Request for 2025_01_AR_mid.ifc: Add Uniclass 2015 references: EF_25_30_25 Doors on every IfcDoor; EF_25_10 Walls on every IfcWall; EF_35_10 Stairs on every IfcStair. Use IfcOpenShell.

First a look at what the model holds.

```python
import ifcopenshell

model = ifcopenshell.open("2025_01_AR_mid.ifc")
print(model.schema)
print("classifications:", [c.Name for c in model.by_type("IfcClassification")])
for ifc_class in ("IfcDoor", "IfcRoof", "IfcStair", "IfcWall", "IfcWindow"):
    print(ifc_class, len(model.by_type(ifc_class)))
```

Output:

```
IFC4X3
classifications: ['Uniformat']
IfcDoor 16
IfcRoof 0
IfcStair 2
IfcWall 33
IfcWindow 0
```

```python
import ifcopenshell
import ifcopenshell.api.classification

model = ifcopenshell.open("2025_01_AR_mid.ifc")

system = ifcopenshell.api.classification.add_classification(model, classification="Uniclass 2015")

codes = {
    "IfcDoor": ("EF_25_30_25", "Doors"),
    "IfcWall": ("EF_25_10", "Walls"),
    "IfcStair": ("EF_35_10", "Stairs"),
}
for ifc_class, (code, name) in codes.items():
    products = model.by_type(ifc_class)
    ifcopenshell.api.classification.add_reference(
        model, products=products, classification=system, identification=code, name=name
    )
    print(code, len(products))

model.write("2025_01_AR_mid_edited.ifc")
```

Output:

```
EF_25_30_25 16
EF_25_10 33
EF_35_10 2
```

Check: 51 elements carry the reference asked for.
